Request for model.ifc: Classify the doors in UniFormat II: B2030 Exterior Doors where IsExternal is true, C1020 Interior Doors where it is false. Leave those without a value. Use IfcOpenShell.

First a look at what the model holds.

```python
import ifcopenshell
import ifcopenshell.util.element

model = ifcopenshell.open("model.ifc")
print(model.schema)
print("classifications:", [c.Name for c in model.by_type("IfcClassification")])
values = [ifcopenshell.util.element.get_pset(e, "Pset_DoorCommon", "IsExternal") for e in model.by_type("IfcDoor")]
for value in (True, False, None):
    print("IsExternal", value, values.count(value))
```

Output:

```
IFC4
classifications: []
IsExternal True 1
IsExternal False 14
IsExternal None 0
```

```python
import ifcopenshell
import ifcopenshell.api.classification
import ifcopenshell.util.element

model = ifcopenshell.open("model.ifc")

system = ifcopenshell.api.classification.add_classification(model, classification="UniFormat II")

doors = model.by_type("IfcDoor")
external = {e: ifcopenshell.util.element.get_pset(e, "Pset_DoorCommon", "IsExternal") for e in doors}
for flag, code, name in ((True, "B2030", "Exterior Doors"), (False, "C1020", "Interior Doors")):
    products = [e for e in doors if external[e] is flag]
    ifcopenshell.api.classification.add_reference(
        model, products=products, classification=system, identification=code, name=name
    )
    print(code, len(products))

model.write("model_edited.ifc")
```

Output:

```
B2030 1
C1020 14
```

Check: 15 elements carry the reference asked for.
